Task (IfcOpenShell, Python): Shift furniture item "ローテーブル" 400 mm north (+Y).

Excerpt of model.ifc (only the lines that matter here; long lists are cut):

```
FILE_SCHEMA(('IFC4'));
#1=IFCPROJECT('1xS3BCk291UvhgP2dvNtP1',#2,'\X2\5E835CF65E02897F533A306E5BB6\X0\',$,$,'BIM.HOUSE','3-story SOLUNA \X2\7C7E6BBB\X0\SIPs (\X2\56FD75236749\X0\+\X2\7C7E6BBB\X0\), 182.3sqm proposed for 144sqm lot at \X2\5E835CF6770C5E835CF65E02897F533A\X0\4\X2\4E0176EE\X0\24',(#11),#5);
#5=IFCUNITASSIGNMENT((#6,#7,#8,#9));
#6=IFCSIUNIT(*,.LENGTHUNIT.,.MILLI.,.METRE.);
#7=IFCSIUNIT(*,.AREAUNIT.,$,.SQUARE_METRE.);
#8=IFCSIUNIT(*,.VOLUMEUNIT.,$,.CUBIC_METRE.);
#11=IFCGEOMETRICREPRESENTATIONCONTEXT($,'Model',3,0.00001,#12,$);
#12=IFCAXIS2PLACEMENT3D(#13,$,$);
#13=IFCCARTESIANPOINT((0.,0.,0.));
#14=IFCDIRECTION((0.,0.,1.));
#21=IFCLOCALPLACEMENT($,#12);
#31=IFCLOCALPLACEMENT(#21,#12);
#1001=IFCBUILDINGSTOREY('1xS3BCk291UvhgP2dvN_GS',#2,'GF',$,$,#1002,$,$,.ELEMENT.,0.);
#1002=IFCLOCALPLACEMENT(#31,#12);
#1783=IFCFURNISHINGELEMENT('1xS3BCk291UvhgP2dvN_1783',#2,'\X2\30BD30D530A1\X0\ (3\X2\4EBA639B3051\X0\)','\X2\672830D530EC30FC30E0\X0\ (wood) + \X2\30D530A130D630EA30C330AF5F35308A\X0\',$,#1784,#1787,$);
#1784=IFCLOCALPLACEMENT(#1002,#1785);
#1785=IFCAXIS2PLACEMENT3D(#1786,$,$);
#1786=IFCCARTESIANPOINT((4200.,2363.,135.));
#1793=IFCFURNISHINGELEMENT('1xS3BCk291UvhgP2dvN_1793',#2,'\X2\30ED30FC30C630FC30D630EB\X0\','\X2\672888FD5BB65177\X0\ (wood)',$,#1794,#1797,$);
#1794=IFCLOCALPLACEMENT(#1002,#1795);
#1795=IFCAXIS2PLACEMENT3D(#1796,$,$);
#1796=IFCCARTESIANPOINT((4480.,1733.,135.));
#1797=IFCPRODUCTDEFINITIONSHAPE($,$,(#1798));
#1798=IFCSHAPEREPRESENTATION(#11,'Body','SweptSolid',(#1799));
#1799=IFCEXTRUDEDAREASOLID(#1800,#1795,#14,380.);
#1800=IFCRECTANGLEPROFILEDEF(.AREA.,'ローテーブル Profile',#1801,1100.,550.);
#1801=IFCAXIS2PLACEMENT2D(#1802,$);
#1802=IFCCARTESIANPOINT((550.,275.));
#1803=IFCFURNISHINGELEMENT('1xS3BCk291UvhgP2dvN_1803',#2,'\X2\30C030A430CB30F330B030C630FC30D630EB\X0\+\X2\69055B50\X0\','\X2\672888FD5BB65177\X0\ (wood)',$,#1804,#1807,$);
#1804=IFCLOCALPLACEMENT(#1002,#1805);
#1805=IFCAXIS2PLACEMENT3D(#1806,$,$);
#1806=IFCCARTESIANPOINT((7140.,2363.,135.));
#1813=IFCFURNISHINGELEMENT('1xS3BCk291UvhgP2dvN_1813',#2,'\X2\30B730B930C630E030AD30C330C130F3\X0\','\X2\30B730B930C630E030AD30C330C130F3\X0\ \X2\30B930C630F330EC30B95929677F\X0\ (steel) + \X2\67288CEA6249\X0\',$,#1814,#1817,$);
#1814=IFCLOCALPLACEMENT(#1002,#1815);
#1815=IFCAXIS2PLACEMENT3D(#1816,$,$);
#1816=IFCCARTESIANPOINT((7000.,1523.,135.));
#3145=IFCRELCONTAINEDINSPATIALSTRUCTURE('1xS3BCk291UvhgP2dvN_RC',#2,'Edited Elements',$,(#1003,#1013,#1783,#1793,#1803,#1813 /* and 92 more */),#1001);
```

```python
import ifcopenshell
import ifcopenshell.api.geometry
import ifcopenshell.util.placement
import ifcopenshell.util.unit

model = ifcopenshell.open("model.ifc")
unit_scale = ifcopenshell.util.unit.calculate_unit_scale(model)

item = model.by_guid("1xS3BCk291UvhgP2dvN_1793")
matrix = ifcopenshell.util.placement.get_local_placement(item.ObjectPlacement)
matrix[1, 3] += 0.4 / unit_scale
ifcopenshell.api.geometry.edit_object_placement(model, product=item, matrix=matrix, is_si=False)

print(ifcopenshell.util.placement.get_local_placement(item.ObjectPlacement).round(3) + 0.0)

model.write("model_edited.ifc")
```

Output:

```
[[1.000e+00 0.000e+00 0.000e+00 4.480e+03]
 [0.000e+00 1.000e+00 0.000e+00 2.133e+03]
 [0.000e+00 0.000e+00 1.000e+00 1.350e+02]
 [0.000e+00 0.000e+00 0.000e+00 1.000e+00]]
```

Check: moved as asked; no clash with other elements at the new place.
